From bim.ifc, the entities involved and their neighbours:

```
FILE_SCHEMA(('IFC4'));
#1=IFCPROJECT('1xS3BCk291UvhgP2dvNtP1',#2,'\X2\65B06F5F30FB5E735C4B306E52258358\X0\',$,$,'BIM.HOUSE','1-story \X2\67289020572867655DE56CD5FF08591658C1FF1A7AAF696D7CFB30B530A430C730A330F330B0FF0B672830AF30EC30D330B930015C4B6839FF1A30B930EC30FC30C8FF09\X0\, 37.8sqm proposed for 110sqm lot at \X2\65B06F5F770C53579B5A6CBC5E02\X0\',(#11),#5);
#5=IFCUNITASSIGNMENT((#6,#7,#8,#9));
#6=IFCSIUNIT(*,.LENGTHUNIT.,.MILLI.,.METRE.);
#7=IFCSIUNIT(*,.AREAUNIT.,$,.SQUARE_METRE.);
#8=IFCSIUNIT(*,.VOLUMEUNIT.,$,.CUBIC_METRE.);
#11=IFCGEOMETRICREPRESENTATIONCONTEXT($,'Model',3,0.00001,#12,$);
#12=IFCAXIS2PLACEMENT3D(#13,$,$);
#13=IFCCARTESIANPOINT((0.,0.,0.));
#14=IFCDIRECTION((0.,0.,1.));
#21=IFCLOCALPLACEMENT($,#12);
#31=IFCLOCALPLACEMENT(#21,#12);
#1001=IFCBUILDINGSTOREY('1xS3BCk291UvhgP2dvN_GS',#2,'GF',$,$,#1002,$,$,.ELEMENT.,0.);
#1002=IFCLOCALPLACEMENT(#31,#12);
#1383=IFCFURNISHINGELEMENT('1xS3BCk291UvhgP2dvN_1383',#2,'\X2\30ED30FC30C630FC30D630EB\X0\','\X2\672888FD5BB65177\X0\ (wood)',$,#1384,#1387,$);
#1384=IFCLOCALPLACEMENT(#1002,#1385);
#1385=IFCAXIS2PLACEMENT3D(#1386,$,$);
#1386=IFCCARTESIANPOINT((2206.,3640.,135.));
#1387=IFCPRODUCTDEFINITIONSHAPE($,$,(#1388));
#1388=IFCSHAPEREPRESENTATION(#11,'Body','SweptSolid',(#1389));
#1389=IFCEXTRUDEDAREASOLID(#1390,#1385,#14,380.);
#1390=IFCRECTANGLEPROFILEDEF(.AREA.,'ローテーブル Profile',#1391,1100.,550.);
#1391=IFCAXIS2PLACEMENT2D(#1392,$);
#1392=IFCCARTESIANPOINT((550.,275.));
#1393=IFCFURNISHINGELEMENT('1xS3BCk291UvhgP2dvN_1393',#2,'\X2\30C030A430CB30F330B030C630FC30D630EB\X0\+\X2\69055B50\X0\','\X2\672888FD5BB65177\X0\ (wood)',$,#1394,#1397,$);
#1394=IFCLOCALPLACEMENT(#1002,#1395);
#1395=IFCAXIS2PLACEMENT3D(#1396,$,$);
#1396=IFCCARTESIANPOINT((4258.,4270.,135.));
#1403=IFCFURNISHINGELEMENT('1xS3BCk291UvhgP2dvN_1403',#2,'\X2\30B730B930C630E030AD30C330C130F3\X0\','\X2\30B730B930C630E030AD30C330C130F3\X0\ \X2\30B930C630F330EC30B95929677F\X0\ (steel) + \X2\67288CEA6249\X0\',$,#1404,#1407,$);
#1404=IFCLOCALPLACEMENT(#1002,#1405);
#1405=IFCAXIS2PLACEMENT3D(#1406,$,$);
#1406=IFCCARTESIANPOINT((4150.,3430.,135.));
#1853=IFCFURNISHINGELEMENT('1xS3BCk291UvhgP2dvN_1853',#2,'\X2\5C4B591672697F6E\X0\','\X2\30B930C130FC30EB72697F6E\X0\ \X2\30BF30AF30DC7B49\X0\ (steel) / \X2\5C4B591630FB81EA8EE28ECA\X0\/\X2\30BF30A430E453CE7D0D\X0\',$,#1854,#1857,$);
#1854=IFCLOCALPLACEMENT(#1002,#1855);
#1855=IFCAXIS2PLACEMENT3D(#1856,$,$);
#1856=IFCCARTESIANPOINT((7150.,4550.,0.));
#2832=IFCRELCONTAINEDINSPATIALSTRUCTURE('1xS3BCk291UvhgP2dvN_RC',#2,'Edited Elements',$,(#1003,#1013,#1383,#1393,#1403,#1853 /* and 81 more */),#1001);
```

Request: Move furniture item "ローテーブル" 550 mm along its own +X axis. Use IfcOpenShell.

```python
import ifcopenshell
import ifcopenshell.api.geometry
import ifcopenshell.util.placement
import ifcopenshell.util.unit

model = ifcopenshell.open("bim.ifc")
unit_scale = ifcopenshell.util.unit.calculate_unit_scale(model)

item = model.by_guid("1xS3BCk291UvhgP2dvN_1383")
matrix = ifcopenshell.util.placement.get_local_placement(item.ObjectPlacement)
matrix[:3, 3] += matrix[:3, 0] * 0.55 / unit_scale
ifcopenshell.api.geometry.edit_object_placement(model, product=item, matrix=matrix, is_si=False)

print(ifcopenshell.util.placement.get_local_placement(item.ObjectPlacement).round(3) + 0.0)

model.write("bim-out.ifc")
```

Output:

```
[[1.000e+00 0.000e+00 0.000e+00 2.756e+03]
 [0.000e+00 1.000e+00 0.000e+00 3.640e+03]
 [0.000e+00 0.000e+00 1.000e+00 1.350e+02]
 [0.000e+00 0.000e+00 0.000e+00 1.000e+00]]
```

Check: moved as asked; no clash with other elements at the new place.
